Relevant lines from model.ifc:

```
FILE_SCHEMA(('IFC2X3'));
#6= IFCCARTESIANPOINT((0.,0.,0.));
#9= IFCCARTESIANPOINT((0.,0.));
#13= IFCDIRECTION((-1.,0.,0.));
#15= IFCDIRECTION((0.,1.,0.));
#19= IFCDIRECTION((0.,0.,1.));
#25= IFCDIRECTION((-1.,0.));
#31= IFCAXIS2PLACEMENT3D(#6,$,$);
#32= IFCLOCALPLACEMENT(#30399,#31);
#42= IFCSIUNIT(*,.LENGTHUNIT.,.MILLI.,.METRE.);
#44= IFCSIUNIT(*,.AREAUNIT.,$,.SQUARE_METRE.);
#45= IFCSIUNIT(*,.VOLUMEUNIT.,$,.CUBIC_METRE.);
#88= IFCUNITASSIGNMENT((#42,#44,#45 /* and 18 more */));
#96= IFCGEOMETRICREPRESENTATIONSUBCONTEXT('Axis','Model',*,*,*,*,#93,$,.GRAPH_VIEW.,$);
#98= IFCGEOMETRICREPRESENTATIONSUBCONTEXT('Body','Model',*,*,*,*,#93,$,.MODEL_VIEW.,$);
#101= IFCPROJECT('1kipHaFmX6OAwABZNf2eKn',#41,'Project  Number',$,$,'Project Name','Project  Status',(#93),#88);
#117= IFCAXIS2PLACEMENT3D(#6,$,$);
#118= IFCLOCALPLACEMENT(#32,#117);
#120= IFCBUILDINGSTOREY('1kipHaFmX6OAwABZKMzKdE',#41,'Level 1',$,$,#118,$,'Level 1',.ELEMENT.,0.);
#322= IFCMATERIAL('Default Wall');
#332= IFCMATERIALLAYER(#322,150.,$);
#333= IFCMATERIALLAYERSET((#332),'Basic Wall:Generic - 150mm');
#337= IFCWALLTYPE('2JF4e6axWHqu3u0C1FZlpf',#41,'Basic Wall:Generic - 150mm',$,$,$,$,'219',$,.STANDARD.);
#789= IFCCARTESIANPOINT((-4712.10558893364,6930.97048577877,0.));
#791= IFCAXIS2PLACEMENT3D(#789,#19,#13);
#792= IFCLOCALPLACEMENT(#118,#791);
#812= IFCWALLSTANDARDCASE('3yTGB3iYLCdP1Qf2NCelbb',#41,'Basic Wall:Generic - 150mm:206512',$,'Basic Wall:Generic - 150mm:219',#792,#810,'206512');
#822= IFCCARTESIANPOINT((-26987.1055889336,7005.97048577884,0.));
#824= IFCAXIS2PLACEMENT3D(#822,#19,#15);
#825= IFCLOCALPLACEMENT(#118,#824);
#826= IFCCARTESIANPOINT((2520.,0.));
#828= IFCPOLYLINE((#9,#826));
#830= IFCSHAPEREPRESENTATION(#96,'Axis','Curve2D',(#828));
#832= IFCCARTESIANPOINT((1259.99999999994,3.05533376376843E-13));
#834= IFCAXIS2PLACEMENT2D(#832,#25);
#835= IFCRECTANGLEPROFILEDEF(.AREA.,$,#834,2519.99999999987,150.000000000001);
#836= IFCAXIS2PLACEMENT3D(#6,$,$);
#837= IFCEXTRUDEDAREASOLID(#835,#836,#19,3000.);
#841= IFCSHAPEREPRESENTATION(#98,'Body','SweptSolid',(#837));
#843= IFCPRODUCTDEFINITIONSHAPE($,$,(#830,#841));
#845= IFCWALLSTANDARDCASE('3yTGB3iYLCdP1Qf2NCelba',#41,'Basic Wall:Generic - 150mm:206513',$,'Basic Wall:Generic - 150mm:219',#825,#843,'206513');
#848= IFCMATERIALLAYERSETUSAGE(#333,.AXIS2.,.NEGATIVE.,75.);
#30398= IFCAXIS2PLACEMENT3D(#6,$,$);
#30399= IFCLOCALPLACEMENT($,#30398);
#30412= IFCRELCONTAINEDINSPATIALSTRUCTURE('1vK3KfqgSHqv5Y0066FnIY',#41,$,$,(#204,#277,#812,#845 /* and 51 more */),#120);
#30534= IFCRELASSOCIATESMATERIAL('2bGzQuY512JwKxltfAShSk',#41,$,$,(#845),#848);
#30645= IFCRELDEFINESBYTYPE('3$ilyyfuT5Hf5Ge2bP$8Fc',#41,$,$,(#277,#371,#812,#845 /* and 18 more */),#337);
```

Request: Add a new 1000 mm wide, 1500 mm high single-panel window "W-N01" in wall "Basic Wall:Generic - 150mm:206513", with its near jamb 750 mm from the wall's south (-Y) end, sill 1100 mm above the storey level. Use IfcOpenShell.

```python
import numpy as np
import ifcopenshell
import ifcopenshell.api.feature
import ifcopenshell.api.geometry
import ifcopenshell.api.root
import ifcopenshell.api.spatial
import ifcopenshell.api.type
import ifcopenshell.geom
import ifcopenshell.util.element
import ifcopenshell.util.placement
import ifcopenshell.util.representation
import ifcopenshell.util.shape
import ifcopenshell.util.unit

model = ifcopenshell.open("model.ifc")
unit_scale = ifcopenshell.util.unit.calculate_unit_scale(model)
settings = ifcopenshell.geom.settings()


def volume(element):
    """Net volume in cubic metres, openings subtracted."""
    shape = ifcopenshell.geom.create_shape(settings, element)
    return ifcopenshell.util.shape.get_volume(shape.geometry)


wall = model.by_guid("3yTGB3iYLCdP1Qf2NCelba")
storey = ifcopenshell.util.element.get_container(wall, ifc_class="IfcBuildingStorey")
context = ifcopenshell.util.representation.get_context(model, "Model", "Body", "MODEL_VIEW")
before = volume(wall)

width, height, from_end, sill = 1, 1.5, 0.75, 1.1  # metres

# The wall runs along its own X axis, and the end named is its -X end.
wall_shape = ifcopenshell.geom.create_shape(settings, wall)
x, y, z = ifcopenshell.util.shape.get_vertices(wall_shape.geometry).T
start = x.min() + from_end
face, thickness = float(y.min()), float(y.max() - y.min())
wall_matrix = ifcopenshell.util.placement.get_local_placement(wall.ObjectPlacement)
level = ifcopenshell.util.placement.get_local_placement(storey.ObjectPlacement)[2, 3]


def in_wall(x, y):
    """Placement at x, y metres in the wall's axes, at sill height."""
    matrix = wall_matrix.copy()
    matrix[:, 3] = wall_matrix @ np.array([x / unit_scale, y / unit_scale, 0.0, 1.0])
    matrix[2, 3] = level + sill / unit_scale
    return matrix


# Opening: a box that overshoots both wall faces by 50 mm.
opening = ifcopenshell.api.root.create_entity(model, ifc_class="IfcOpeningElement")
box = ifcopenshell.api.geometry.add_wall_representation(
    model, context=context, length=width, height=height, thickness=thickness + 0.1
)
ifcopenshell.api.geometry.assign_representation(model, product=opening, representation=box)
ifcopenshell.api.geometry.edit_object_placement(model, product=opening, matrix=in_wall(start, face - 0.05), is_si=False)
ifcopenshell.api.feature.add_feature(model, feature=opening, element=wall)

window = ifcopenshell.api.root.create_entity(model, ifc_class="IfcWindow", name="W-N01")
window.OverallWidth, window.OverallHeight = width / unit_scale, height / unit_scale
body = ifcopenshell.api.geometry.add_window_representation(
    model,
    context=context,
    overall_width=window.OverallWidth,
    overall_height=window.OverallHeight,
    partition_type="SINGLE_PANEL",
)
ifcopenshell.api.geometry.assign_representation(model, product=window, representation=body)
ifcopenshell.api.spatial.assign_container(model, products=[window], relating_structure=storey)
fills = ifcopenshell.api.feature.add_filling(model, opening=opening, element=window)
fills.OwnerHistory = window.OwnerHistory  # required in IFC2X3

# IFC2X3 keeps the operation on the window style.
style = ifcopenshell.api.root.create_entity(model, ifc_class="IfcWindowStyle", name="W-N01")
style.OperationType, style.ConstructionType = "SINGLE_PANEL", "NOTDEFINED"
style.ParameterTakesPrecedence = style.Sizeable = False
ifcopenshell.api.type.assign_type(model, related_objects=[window], relating_type=style)

# Centre the window in the wall's thickness.
ifcopenshell.api.geometry.edit_object_placement(model, product=window, matrix=in_wall(start, face), is_si=False)
window_shape = ifcopenshell.geom.create_shape(settings, window)
depth = ifcopenshell.util.shape.get_vertices(window_shape.geometry)[:, 1]
offset = face + thickness / 2 - (depth.min() + depth.max()) / 2
ifcopenshell.api.geometry.edit_object_placement(model, product=window, matrix=in_wall(start, offset), is_si=False)

after = volume(wall)

print(f"wall volume {before:.3f} -> {after:.3f} m3")

model.write("model_edited.ifc")
```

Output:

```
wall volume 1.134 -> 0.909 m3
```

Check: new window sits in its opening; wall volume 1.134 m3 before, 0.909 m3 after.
